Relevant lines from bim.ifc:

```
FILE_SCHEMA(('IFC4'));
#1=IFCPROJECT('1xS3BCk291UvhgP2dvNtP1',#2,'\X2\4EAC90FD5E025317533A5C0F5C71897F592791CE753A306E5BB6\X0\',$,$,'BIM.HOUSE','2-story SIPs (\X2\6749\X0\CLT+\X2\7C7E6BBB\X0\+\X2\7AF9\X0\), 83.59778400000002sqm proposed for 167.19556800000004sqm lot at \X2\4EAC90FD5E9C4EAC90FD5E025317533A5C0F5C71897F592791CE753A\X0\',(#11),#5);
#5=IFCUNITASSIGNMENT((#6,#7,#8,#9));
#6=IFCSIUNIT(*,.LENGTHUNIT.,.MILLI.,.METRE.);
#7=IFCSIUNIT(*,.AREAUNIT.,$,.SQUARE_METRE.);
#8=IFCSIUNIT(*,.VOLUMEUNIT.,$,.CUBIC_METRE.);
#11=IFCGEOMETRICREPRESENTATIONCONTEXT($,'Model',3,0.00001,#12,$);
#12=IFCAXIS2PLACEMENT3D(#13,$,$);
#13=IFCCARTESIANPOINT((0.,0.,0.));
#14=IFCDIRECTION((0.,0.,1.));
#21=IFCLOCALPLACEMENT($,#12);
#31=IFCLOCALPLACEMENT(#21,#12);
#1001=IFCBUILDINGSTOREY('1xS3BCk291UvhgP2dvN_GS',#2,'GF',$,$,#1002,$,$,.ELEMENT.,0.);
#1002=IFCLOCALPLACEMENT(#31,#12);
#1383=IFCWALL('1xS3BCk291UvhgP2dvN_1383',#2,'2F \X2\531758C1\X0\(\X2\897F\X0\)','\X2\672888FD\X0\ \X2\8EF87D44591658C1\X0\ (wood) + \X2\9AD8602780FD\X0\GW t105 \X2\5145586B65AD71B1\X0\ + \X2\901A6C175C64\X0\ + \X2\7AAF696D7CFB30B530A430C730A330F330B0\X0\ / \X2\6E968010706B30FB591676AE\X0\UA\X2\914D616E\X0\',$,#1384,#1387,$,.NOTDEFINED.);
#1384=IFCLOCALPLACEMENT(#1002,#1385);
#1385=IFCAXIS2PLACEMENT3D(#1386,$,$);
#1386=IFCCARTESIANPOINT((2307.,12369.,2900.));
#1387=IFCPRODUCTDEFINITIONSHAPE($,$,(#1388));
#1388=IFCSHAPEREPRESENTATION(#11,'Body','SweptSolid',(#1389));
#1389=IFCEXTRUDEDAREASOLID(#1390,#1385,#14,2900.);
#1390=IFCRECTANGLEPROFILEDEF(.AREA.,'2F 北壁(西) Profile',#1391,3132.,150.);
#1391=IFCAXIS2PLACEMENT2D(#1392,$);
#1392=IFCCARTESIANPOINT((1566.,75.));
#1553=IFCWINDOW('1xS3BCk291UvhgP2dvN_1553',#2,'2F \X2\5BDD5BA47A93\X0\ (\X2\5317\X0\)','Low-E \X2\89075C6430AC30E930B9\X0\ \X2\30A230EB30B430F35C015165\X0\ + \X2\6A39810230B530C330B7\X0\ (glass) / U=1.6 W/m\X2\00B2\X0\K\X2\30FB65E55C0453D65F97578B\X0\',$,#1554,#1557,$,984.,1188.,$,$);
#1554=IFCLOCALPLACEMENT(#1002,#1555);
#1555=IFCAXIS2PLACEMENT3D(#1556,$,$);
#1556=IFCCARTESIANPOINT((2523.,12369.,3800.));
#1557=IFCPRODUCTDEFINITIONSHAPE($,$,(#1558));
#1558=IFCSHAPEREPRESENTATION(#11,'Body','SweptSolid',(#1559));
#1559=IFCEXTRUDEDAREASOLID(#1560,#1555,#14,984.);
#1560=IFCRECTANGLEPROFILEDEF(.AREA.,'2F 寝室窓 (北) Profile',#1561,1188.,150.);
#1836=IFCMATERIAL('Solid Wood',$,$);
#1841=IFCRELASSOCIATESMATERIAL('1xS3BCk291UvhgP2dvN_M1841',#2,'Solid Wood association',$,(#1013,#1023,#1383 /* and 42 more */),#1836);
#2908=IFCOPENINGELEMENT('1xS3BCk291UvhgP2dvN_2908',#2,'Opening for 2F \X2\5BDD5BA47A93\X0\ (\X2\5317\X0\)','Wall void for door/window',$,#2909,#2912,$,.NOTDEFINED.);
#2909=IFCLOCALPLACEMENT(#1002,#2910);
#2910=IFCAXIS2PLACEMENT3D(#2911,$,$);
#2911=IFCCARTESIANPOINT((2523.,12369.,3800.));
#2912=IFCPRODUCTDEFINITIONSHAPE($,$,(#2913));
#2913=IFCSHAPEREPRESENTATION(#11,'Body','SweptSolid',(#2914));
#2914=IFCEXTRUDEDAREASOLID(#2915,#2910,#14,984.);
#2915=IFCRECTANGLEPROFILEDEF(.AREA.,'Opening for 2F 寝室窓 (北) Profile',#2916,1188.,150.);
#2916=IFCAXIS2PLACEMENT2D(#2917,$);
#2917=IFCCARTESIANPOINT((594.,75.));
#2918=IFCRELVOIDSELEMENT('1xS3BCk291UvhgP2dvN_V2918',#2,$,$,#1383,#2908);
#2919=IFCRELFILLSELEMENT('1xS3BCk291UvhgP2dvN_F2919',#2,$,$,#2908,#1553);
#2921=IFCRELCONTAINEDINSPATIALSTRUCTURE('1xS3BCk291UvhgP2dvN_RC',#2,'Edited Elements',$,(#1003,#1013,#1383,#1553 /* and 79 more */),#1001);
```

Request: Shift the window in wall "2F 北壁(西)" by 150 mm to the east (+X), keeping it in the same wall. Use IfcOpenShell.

```python
import ifcopenshell
import ifcopenshell.api.geometry
import ifcopenshell.util.placement
import ifcopenshell.util.unit

model = ifcopenshell.open("bim.ifc")
unit_scale = ifcopenshell.util.unit.calculate_unit_scale(model)

window = model.by_id(1553)
opening = window.FillsVoids[0].RelatingOpeningElement
wall = opening.VoidsElements[0].RelatingBuildingElement

wall_matrix = ifcopenshell.util.placement.get_local_placement(wall.ObjectPlacement)
shift = wall_matrix[:3, 0] * 0.15 / unit_scale
before = ifcopenshell.util.placement.get_local_placement(window.ObjectPlacement)[:3, 3].copy()

# The window is not placed relative to its opening, so move both.
for product in (opening, window):
    matrix = ifcopenshell.util.placement.get_local_placement(product.ObjectPlacement)
    matrix[:3, 3] += shift
    ifcopenshell.api.geometry.edit_object_placement(model, product=product, matrix=matrix, is_si=False)

after = ifcopenshell.util.placement.get_local_placement(window.ObjectPlacement)[:3, 3]
print("window moved by", (after - before).round(3) + 0.0)

model.write("bim_edited.ifc")
```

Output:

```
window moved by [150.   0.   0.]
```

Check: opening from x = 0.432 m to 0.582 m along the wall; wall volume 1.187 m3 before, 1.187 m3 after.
